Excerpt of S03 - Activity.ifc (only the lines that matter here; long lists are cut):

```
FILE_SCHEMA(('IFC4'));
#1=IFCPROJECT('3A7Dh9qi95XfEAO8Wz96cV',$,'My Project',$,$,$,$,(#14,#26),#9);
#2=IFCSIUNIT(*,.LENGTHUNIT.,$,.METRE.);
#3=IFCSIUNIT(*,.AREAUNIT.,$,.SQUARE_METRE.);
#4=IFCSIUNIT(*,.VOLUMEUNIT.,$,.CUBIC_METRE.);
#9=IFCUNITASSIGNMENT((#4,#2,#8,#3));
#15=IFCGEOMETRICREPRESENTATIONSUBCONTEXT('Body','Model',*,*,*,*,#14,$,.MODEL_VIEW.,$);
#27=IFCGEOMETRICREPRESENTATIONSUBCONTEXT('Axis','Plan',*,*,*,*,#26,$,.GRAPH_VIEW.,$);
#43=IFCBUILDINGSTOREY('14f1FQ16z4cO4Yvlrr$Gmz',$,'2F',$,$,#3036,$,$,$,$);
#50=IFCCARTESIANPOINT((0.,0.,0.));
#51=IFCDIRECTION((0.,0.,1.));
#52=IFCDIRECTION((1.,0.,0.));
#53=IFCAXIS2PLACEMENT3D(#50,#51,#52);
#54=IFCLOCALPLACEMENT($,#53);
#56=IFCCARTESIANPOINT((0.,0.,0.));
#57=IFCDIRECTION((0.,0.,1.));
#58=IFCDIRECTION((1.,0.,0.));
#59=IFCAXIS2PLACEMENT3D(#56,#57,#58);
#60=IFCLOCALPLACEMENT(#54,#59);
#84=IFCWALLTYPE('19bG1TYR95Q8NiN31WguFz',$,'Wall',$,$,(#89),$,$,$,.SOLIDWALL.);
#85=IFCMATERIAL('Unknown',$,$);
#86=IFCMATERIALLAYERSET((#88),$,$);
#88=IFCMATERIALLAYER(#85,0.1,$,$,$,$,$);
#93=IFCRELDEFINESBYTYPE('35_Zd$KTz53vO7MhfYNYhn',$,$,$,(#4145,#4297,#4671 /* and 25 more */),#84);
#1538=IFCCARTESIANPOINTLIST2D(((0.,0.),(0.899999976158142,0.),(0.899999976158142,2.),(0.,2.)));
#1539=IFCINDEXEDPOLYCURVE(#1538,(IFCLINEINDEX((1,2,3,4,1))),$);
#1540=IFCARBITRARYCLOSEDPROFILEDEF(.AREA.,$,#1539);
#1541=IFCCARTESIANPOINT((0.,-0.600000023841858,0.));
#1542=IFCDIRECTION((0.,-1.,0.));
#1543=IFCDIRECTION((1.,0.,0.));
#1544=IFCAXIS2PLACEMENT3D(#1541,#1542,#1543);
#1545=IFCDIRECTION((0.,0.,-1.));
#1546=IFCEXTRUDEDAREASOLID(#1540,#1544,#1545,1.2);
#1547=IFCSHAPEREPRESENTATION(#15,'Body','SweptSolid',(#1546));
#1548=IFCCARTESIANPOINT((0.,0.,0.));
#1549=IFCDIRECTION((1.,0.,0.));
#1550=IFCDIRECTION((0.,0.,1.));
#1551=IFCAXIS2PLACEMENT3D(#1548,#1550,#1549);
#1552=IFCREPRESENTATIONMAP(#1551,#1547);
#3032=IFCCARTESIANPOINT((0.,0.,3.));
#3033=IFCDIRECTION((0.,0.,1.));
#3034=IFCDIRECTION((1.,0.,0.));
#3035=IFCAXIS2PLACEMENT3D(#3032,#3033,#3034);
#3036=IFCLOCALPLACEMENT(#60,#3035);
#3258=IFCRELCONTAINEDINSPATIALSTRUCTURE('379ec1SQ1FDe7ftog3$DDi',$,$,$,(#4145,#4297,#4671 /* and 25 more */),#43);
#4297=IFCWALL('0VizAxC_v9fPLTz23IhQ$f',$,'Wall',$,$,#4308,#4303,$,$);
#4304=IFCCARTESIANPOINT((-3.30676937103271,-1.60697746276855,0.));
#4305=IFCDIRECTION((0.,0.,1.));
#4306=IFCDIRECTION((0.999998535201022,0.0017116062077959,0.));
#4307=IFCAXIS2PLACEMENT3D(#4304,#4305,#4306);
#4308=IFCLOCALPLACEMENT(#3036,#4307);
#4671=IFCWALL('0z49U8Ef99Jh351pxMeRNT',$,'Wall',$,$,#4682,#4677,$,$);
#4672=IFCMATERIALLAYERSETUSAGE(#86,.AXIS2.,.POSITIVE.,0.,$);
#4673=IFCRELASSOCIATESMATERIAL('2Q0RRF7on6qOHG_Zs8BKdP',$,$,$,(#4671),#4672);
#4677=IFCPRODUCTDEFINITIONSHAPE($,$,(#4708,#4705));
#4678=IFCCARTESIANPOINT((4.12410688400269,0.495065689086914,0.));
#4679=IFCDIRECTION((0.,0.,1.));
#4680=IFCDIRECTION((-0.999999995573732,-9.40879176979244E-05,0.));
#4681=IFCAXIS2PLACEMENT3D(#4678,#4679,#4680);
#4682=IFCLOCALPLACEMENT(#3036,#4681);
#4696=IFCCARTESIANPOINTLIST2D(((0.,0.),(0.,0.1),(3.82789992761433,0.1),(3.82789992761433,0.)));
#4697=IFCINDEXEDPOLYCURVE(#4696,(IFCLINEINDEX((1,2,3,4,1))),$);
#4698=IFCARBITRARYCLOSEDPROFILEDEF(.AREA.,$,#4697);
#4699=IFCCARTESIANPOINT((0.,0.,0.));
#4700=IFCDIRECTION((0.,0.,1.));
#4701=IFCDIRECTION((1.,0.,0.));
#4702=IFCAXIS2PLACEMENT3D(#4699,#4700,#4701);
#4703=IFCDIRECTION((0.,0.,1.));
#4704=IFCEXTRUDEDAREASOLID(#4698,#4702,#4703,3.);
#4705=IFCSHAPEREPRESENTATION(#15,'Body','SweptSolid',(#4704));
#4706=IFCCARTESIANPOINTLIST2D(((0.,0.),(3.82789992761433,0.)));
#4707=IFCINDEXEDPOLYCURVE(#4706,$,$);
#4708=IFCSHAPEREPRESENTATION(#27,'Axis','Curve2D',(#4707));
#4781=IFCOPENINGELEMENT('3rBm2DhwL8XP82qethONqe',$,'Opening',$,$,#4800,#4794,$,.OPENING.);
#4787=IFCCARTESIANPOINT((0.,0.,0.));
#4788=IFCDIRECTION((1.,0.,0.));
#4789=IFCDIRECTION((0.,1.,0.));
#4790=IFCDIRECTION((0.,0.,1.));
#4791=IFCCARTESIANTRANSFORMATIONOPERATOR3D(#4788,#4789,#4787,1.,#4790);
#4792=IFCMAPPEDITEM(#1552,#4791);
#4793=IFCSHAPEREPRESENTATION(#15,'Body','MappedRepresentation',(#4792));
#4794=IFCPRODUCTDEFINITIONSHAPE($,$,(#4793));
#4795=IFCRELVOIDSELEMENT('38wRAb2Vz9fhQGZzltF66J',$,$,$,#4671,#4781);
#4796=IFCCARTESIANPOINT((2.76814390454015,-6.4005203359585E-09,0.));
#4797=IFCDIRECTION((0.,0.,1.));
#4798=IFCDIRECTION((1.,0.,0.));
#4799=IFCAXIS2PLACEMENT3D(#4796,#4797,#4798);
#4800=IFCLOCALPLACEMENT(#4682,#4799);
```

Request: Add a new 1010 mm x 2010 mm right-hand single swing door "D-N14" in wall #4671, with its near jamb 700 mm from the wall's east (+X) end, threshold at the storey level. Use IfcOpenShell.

```python
import numpy as np
import ifcopenshell
import ifcopenshell.api.feature
import ifcopenshell.api.geometry
import ifcopenshell.api.root
import ifcopenshell.api.spatial
import ifcopenshell.geom
import ifcopenshell.util.element
import ifcopenshell.util.placement
import ifcopenshell.util.representation
import ifcopenshell.util.shape
import ifcopenshell.util.unit

model = ifcopenshell.open("S03 - Activity.ifc")
unit_scale = ifcopenshell.util.unit.calculate_unit_scale(model)
settings = ifcopenshell.geom.settings()


def volume(element):
    """Net volume in cubic metres, openings subtracted."""
    shape = ifcopenshell.geom.create_shape(settings, element)
    return ifcopenshell.util.shape.get_volume(shape.geometry)


wall = model.by_id(4671)
storey = ifcopenshell.util.element.get_container(wall, ifc_class="IfcBuildingStorey")
context = ifcopenshell.util.representation.get_context(model, "Model", "Body", "MODEL_VIEW")
before = volume(wall)

width, height, from_end, sill = 1.01, 2.01, 0.7, 0.0  # metres

# The wall runs along its own X axis, and the end named is its -X end.
wall_shape = ifcopenshell.geom.create_shape(settings, wall)
x, y, z = ifcopenshell.util.shape.get_vertices(wall_shape.geometry).T
start = x.min() + from_end
face, thickness = float(y.min()), float(y.max() - y.min())
wall_matrix = ifcopenshell.util.placement.get_local_placement(wall.ObjectPlacement)
level = ifcopenshell.util.placement.get_local_placement(storey.ObjectPlacement)[2, 3]


def in_wall(x, y):
    """Placement at x, y metres in the wall's axes, at sill height."""
    matrix = wall_matrix.copy()
    matrix[:, 3] = wall_matrix @ np.array([x / unit_scale, y / unit_scale, 0.0, 1.0])
    matrix[2, 3] = level + sill / unit_scale
    return matrix


# Opening: a box that overshoots both wall faces by 50 mm.
opening = ifcopenshell.api.root.create_entity(model, ifc_class="IfcOpeningElement", predefined_type="OPENING")
box = ifcopenshell.api.geometry.add_wall_representation(
    model, context=context, length=width, height=height, thickness=thickness + 0.1
)
ifcopenshell.api.geometry.assign_representation(model, product=opening, representation=box)
ifcopenshell.api.geometry.edit_object_placement(model, product=opening, matrix=in_wall(start, face - 0.05), is_si=False)
ifcopenshell.api.feature.add_feature(model, feature=opening, element=wall)

door = ifcopenshell.api.root.create_entity(model, ifc_class="IfcDoor", name="D-N14", predefined_type="DOOR")
door.OverallWidth, door.OverallHeight = width / unit_scale, height / unit_scale
door.OperationType = "SINGLE_SWING_RIGHT"
body = ifcopenshell.api.geometry.add_door_representation(
    model,
    context=context,
    overall_width=door.OverallWidth,
    overall_height=door.OverallHeight,
    operation_type="SINGLE_SWING_RIGHT",
    lining_properties={"LiningDepth": thickness / unit_scale, "ThresholdDepth": thickness / unit_scale},
)
ifcopenshell.api.geometry.assign_representation(model, product=door, representation=body)
ifcopenshell.api.spatial.assign_container(model, products=[door], relating_structure=storey)
ifcopenshell.api.feature.add_filling(model, opening=opening, element=door)

# The lining spans the wall, so the door starts at the wall face.
ifcopenshell.api.geometry.edit_object_placement(model, product=door, matrix=in_wall(start, face), is_si=False)

after = volume(wall)

print(f"wall volume {before:.3f} -> {after:.3f} m3")

model.write("S03 - Activity_v2.ifc")
```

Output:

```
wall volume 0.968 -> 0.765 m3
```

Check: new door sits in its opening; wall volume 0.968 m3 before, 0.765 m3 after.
